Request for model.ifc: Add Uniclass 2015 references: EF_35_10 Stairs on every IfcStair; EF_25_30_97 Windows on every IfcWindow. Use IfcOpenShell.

First a look at what the model holds.

```python
import ifcopenshell

model = ifcopenshell.open("model.ifc")
print(model.schema)
print("classifications:", [c.Name for c in model.by_type("IfcClassification")])
for ifc_class in ("IfcDoor", "IfcRoof", "IfcStair", "IfcWall", "IfcWindow"):
    print(ifc_class, len(model.by_type(ifc_class)))
```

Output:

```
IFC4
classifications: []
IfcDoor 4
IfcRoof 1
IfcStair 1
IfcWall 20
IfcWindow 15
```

```python
import ifcopenshell
import ifcopenshell.api.classification

model = ifcopenshell.open("model.ifc")

system = ifcopenshell.api.classification.add_classification(model, classification="Uniclass 2015")

codes = {
    "IfcStair": ("EF_35_10", "Stairs"),
    "IfcWindow": ("EF_25_30_97", "Windows"),
}
for ifc_class, (code, name) in codes.items():
    products = model.by_type(ifc_class)
    ifcopenshell.api.classification.add_reference(
        model, products=products, classification=system, identification=code, name=name
    )
    print(code, len(products))

model.write("model_v2.ifc")
```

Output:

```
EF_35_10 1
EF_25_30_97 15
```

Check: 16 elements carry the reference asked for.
